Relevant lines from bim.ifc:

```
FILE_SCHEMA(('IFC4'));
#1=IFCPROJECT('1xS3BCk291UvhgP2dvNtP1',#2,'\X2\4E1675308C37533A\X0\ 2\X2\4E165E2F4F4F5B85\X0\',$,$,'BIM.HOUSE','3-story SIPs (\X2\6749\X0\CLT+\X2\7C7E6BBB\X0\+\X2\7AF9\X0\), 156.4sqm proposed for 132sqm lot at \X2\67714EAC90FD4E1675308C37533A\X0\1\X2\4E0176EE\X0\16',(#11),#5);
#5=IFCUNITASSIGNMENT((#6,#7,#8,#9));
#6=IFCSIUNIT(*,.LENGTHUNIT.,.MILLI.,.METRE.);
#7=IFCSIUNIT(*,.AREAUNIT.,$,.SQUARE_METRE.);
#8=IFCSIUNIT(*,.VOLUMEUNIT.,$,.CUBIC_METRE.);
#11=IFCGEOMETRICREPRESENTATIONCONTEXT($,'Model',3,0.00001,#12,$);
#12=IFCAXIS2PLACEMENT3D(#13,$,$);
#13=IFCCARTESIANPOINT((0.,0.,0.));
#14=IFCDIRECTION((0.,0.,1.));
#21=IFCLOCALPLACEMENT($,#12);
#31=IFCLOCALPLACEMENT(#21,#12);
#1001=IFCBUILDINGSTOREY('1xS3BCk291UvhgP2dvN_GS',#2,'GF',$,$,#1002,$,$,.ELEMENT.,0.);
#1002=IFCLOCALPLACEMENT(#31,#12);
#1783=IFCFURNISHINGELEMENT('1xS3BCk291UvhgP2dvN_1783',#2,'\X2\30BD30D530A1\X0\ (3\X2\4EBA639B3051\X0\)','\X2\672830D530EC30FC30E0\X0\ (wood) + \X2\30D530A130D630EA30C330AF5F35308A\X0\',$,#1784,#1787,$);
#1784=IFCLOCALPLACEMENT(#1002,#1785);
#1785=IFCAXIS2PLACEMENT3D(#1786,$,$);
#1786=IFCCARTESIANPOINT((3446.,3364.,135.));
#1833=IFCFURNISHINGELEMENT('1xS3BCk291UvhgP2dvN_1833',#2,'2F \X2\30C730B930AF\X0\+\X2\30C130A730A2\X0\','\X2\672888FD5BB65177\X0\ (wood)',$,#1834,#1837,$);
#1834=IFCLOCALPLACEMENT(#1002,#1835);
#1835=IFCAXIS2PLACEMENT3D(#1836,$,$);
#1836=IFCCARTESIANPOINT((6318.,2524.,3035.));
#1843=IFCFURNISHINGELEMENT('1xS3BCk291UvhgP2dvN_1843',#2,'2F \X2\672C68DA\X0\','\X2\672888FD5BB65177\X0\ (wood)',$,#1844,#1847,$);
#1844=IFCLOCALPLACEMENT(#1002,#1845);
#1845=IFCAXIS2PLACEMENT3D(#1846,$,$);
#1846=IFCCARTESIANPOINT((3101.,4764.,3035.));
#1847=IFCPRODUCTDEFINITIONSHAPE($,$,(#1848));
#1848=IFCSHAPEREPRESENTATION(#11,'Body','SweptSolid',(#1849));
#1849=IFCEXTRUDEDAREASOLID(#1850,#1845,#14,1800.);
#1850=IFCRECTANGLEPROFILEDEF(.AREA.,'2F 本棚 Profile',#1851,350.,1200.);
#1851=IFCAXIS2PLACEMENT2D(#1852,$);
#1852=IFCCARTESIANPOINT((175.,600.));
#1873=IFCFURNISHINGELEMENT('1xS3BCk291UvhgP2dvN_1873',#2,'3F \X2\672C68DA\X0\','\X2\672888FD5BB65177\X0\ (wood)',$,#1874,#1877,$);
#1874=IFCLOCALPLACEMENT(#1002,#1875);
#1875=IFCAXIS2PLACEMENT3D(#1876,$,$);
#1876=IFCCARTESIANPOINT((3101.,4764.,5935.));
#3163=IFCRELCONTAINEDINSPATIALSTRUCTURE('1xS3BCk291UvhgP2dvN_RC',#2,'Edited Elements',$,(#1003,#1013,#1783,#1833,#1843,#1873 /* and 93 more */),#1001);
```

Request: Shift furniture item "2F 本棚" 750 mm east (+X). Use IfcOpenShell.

```python
import ifcopenshell
import ifcopenshell.api.geometry
import ifcopenshell.util.placement

model = ifcopenshell.open("bim.ifc")

item = model.by_id(1843)
matrix = ifcopenshell.util.placement.get_local_placement(item.ObjectPlacement)
matrix[0, 3] += 750.0
ifcopenshell.api.geometry.edit_object_placement(model, product=item, matrix=matrix, is_si=False)

print(ifcopenshell.util.placement.get_local_placement(item.ObjectPlacement).round(3) + 0.0)

model.write("bim_rev.ifc")
```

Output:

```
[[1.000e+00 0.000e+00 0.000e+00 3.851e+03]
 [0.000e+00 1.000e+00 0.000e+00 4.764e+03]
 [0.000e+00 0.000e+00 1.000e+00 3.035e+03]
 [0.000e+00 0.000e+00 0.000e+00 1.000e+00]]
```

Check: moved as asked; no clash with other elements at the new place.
